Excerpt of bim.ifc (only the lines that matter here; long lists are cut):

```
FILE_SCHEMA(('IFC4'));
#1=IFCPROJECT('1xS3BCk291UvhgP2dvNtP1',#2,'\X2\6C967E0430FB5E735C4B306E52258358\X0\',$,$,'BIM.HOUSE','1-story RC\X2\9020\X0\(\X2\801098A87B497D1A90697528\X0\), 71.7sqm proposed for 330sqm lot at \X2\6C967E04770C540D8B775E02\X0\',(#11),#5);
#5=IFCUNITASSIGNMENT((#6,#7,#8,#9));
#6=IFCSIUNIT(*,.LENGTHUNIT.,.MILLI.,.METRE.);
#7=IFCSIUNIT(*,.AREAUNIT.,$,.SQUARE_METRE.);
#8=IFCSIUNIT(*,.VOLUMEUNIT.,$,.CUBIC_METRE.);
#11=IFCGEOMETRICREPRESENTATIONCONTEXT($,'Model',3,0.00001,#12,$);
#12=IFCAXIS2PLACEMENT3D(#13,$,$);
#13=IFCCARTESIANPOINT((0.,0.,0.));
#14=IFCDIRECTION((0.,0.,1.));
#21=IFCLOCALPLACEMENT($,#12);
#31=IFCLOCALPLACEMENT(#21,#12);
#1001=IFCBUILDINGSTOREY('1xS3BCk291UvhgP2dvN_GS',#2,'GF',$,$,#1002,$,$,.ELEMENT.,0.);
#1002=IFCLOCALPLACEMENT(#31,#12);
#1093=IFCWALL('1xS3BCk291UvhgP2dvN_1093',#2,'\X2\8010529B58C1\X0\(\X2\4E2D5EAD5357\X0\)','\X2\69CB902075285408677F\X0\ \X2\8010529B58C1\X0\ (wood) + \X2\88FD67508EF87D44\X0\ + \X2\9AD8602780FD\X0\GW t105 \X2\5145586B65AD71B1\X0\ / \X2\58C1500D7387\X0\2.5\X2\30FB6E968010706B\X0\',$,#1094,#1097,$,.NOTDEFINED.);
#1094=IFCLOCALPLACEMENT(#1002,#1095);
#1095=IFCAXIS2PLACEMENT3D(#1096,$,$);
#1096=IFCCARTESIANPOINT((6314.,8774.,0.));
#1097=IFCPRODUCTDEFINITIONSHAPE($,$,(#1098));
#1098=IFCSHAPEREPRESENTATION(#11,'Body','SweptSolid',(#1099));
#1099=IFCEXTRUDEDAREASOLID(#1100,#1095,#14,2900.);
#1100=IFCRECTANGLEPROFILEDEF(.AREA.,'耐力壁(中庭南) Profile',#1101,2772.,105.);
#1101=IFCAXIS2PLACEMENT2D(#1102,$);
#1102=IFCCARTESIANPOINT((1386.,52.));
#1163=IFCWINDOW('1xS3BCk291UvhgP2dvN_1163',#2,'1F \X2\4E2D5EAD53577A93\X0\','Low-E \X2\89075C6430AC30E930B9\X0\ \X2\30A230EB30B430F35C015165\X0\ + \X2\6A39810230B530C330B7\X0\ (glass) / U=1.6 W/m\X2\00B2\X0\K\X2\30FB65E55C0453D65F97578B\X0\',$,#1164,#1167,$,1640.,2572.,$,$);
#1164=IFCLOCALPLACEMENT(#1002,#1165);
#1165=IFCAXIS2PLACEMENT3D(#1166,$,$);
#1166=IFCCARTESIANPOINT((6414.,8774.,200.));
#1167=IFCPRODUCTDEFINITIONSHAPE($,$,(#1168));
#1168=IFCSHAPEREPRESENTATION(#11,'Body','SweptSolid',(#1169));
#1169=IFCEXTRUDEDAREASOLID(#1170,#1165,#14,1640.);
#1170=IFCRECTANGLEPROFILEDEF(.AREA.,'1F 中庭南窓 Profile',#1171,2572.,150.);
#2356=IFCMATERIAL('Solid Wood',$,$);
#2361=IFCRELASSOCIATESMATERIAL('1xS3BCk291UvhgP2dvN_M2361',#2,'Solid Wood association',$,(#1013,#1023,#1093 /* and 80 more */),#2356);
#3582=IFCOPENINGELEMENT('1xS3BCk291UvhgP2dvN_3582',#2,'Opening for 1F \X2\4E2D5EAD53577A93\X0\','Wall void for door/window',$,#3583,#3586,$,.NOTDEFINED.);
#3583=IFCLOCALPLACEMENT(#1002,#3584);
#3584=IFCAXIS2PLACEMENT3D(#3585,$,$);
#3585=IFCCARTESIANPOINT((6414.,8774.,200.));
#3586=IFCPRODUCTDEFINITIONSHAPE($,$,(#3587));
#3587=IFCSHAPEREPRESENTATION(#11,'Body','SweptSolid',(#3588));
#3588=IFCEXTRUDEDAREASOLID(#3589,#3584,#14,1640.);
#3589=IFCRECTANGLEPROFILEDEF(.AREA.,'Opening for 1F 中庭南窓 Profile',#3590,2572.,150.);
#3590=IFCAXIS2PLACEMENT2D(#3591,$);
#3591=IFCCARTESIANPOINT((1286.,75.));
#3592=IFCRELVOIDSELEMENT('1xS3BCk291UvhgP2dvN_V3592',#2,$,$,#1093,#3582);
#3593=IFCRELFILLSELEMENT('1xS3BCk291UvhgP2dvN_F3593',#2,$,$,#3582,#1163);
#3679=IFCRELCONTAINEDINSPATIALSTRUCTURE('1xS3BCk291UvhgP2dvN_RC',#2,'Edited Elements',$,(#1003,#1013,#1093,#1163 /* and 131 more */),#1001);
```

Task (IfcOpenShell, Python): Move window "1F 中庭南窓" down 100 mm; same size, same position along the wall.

```python
import numpy as np
import ifcopenshell
import ifcopenshell.api.geometry
import ifcopenshell.util.placement
import ifcopenshell.util.unit

model = ifcopenshell.open("bim.ifc")
unit_scale = ifcopenshell.util.unit.calculate_unit_scale(model)

window = model.by_id(1163)
opening = window.FillsVoids[0].RelatingOpeningElement
dz = -100.0

shift = np.array([0.0, 0.0, dz])
# The window is not placed relative to its opening, so move both.
for product in (opening, window):
    matrix = ifcopenshell.util.placement.get_local_placement(product.ObjectPlacement)
    matrix[:3, 3] += shift
    ifcopenshell.api.geometry.edit_object_placement(model, product=product, matrix=matrix, is_si=False)

print(f"moved by {dz * unit_scale:+.3f} m")

model.write("bim_edited.ifc")
```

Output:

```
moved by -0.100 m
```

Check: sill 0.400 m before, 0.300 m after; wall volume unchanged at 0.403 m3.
